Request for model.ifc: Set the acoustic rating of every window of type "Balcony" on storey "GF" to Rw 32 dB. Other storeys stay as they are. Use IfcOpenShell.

First a look at what the model holds.

```python
import ifcopenshell
import ifcopenshell.util.element

model = ifcopenshell.open("model.ifc")
print(model.schema)
storey = next(s for s in model.by_type("IfcBuildingStorey") if s.Name == "GF")
windows = [e for e in ifcopenshell.util.element.get_decomposition(storey) if e.is_a("IfcWindow")]
seen = {}
for e in windows:
    element_type = ifcopenshell.util.element.get_type(e)
    key = (element_type.Name if element_type != e and element_type else None, ifcopenshell.util.element.get_pset(e, "Pset_WindowCommon", "AcousticRating"))
    seen[key] = seen.get(key, 0) + 1
for (name, value), count in sorted(seen.items(), key=str):
    print(count, "x", name, "|", value)
```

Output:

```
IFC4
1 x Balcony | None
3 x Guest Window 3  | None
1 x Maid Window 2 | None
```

```python
import ifcopenshell
import ifcopenshell.api.pset
import ifcopenshell.util.element

model = ifcopenshell.open("model.ifc")

storey = next(s for s in model.by_type("IfcBuildingStorey") if s.Name == "GF")
windows = [e for e in ifcopenshell.util.element.get_decomposition(storey) if e.is_a("IfcWindow")]

count = 0
for e in windows:
    element_type = ifcopenshell.util.element.get_type(e)
    if element_type in (None, e) or element_type.Name != "Balcony":
        continue
    # add_pset returns the element's existing set when there is one.
    pset = ifcopenshell.api.pset.add_pset(model, product=e, name="Pset_WindowCommon")
    ifcopenshell.api.pset.edit_pset(model, pset=pset, properties={"AcousticRating": "Rw 32 dB"})
    count += 1

print(count, "windows updated")

model.write("model_edited.ifc")
```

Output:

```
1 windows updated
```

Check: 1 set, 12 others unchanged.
